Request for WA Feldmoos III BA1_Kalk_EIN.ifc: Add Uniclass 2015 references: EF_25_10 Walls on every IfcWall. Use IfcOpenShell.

First a look at what the model holds.

```python
import ifcopenshell

model = ifcopenshell.open("WA Feldmoos III BA1_Kalk_EIN.ifc")
print(model.schema)
print("classifications:", [c.Name for c in model.by_type("IfcClassification")])
for ifc_class in ("IfcDoor", "IfcRoof", "IfcStair", "IfcWall", "IfcWindow"):
    print(ifc_class, len(model.by_type(ifc_class)))
```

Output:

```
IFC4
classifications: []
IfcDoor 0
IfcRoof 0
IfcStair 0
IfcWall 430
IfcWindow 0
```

```python
import ifcopenshell
import ifcopenshell.api.classification

model = ifcopenshell.open("WA Feldmoos III BA1_Kalk_EIN.ifc")

system = ifcopenshell.api.classification.add_classification(model, classification="Uniclass 2015")

codes = {
    "IfcWall": ("EF_25_10", "Walls"),
}
for ifc_class, (code, name) in codes.items():
    products = model.by_type(ifc_class)
    ifcopenshell.api.classification.add_reference(
        model, products=products, classification=system, identification=code, name=name
    )
    print(code, len(products))

model.write("WA Feldmoos III BA1_Kalk_EIN_updated.ifc")
```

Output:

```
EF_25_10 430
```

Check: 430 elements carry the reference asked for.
